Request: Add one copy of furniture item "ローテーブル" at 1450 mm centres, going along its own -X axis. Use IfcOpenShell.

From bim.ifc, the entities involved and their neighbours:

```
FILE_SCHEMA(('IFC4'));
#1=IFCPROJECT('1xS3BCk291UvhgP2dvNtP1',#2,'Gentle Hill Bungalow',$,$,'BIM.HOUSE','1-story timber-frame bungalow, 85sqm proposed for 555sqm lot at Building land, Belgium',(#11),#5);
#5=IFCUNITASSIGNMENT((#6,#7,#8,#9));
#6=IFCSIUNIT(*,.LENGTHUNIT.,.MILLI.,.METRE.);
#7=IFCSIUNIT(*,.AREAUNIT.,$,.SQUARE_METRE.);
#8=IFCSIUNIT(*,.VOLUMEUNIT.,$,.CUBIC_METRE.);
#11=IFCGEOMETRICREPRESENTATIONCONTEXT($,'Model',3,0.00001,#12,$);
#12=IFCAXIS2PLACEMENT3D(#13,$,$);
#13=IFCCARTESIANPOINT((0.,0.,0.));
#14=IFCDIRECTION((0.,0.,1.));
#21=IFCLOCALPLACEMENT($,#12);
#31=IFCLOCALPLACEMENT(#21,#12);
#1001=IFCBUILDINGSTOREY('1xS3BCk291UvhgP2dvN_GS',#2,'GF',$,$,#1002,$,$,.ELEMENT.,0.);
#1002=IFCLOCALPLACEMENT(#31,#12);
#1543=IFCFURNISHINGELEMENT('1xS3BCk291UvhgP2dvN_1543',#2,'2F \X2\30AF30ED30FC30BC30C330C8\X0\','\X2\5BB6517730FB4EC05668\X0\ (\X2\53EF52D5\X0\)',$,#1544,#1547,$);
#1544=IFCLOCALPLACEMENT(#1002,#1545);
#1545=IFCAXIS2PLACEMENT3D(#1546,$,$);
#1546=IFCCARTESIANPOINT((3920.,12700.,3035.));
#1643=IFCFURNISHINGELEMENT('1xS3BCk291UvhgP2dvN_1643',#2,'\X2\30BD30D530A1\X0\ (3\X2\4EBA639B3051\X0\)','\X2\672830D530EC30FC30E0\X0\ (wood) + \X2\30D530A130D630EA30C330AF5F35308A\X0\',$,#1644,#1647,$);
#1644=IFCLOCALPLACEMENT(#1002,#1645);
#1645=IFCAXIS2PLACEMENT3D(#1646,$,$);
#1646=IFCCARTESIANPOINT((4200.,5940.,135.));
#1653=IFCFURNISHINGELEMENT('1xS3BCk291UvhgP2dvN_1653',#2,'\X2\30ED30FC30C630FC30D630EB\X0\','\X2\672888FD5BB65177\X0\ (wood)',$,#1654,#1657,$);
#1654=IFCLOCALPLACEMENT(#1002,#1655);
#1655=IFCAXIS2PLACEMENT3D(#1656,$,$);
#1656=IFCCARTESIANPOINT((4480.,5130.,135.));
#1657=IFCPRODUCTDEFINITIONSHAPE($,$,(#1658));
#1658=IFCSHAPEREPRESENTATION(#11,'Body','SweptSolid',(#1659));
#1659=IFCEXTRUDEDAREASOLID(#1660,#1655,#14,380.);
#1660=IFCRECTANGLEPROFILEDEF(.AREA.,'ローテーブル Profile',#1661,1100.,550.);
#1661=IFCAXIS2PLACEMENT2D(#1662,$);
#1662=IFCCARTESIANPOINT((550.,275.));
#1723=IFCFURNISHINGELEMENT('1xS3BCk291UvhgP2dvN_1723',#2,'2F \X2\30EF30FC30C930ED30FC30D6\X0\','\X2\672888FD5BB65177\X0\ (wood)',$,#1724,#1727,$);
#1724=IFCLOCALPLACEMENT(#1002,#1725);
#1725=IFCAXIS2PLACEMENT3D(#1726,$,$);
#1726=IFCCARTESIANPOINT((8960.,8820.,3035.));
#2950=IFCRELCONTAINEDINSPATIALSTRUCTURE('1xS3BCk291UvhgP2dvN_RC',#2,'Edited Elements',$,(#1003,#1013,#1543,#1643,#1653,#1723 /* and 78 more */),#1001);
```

```python
import ifcopenshell
import ifcopenshell.api.geometry
import ifcopenshell.api.root
import ifcopenshell.util.element
import ifcopenshell.util.placement

model = ifcopenshell.open("bim.ifc")


def reuse_history(source, copy):
    """copy_class also copies each property set's owner history, people and application; keep the originals."""
    for rel in copy.IsDefinedBy:
        if rel.is_a("IfcRelDefinesByProperties") and (history := rel.RelatingPropertyDefinition.OwnerHistory):
            rel.RelatingPropertyDefinition.OwnerHistory = source.OwnerHistory
            ifcopenshell.util.element.remove_deep2(model, history)


source = model.by_guid("1xS3BCk291UvhgP2dvN_1653")
base = ifcopenshell.util.placement.get_local_placement(source.ObjectPlacement)
step = -base[:3, 0] * 1450.0

for i in range(1, 2):
    copy = ifcopenshell.api.root.copy_class(model, product=source)
    copy.Representation = ifcopenshell.util.element.copy_deep(
        model, source.Representation, exclude=["IfcGeometricRepresentationContext", "IfcRepresentationMap"]
    )
    reuse_history(source, copy)
    matrix = base.copy()
    matrix[:3, 3] += i * step
    print("added at", matrix[:3, 3].round(3) + 0.0)
    ifcopenshell.api.geometry.edit_object_placement(model, product=copy, matrix=matrix, is_si=False)

model.write("bim_edited.ifc")
```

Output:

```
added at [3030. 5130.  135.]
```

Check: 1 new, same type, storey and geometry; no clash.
